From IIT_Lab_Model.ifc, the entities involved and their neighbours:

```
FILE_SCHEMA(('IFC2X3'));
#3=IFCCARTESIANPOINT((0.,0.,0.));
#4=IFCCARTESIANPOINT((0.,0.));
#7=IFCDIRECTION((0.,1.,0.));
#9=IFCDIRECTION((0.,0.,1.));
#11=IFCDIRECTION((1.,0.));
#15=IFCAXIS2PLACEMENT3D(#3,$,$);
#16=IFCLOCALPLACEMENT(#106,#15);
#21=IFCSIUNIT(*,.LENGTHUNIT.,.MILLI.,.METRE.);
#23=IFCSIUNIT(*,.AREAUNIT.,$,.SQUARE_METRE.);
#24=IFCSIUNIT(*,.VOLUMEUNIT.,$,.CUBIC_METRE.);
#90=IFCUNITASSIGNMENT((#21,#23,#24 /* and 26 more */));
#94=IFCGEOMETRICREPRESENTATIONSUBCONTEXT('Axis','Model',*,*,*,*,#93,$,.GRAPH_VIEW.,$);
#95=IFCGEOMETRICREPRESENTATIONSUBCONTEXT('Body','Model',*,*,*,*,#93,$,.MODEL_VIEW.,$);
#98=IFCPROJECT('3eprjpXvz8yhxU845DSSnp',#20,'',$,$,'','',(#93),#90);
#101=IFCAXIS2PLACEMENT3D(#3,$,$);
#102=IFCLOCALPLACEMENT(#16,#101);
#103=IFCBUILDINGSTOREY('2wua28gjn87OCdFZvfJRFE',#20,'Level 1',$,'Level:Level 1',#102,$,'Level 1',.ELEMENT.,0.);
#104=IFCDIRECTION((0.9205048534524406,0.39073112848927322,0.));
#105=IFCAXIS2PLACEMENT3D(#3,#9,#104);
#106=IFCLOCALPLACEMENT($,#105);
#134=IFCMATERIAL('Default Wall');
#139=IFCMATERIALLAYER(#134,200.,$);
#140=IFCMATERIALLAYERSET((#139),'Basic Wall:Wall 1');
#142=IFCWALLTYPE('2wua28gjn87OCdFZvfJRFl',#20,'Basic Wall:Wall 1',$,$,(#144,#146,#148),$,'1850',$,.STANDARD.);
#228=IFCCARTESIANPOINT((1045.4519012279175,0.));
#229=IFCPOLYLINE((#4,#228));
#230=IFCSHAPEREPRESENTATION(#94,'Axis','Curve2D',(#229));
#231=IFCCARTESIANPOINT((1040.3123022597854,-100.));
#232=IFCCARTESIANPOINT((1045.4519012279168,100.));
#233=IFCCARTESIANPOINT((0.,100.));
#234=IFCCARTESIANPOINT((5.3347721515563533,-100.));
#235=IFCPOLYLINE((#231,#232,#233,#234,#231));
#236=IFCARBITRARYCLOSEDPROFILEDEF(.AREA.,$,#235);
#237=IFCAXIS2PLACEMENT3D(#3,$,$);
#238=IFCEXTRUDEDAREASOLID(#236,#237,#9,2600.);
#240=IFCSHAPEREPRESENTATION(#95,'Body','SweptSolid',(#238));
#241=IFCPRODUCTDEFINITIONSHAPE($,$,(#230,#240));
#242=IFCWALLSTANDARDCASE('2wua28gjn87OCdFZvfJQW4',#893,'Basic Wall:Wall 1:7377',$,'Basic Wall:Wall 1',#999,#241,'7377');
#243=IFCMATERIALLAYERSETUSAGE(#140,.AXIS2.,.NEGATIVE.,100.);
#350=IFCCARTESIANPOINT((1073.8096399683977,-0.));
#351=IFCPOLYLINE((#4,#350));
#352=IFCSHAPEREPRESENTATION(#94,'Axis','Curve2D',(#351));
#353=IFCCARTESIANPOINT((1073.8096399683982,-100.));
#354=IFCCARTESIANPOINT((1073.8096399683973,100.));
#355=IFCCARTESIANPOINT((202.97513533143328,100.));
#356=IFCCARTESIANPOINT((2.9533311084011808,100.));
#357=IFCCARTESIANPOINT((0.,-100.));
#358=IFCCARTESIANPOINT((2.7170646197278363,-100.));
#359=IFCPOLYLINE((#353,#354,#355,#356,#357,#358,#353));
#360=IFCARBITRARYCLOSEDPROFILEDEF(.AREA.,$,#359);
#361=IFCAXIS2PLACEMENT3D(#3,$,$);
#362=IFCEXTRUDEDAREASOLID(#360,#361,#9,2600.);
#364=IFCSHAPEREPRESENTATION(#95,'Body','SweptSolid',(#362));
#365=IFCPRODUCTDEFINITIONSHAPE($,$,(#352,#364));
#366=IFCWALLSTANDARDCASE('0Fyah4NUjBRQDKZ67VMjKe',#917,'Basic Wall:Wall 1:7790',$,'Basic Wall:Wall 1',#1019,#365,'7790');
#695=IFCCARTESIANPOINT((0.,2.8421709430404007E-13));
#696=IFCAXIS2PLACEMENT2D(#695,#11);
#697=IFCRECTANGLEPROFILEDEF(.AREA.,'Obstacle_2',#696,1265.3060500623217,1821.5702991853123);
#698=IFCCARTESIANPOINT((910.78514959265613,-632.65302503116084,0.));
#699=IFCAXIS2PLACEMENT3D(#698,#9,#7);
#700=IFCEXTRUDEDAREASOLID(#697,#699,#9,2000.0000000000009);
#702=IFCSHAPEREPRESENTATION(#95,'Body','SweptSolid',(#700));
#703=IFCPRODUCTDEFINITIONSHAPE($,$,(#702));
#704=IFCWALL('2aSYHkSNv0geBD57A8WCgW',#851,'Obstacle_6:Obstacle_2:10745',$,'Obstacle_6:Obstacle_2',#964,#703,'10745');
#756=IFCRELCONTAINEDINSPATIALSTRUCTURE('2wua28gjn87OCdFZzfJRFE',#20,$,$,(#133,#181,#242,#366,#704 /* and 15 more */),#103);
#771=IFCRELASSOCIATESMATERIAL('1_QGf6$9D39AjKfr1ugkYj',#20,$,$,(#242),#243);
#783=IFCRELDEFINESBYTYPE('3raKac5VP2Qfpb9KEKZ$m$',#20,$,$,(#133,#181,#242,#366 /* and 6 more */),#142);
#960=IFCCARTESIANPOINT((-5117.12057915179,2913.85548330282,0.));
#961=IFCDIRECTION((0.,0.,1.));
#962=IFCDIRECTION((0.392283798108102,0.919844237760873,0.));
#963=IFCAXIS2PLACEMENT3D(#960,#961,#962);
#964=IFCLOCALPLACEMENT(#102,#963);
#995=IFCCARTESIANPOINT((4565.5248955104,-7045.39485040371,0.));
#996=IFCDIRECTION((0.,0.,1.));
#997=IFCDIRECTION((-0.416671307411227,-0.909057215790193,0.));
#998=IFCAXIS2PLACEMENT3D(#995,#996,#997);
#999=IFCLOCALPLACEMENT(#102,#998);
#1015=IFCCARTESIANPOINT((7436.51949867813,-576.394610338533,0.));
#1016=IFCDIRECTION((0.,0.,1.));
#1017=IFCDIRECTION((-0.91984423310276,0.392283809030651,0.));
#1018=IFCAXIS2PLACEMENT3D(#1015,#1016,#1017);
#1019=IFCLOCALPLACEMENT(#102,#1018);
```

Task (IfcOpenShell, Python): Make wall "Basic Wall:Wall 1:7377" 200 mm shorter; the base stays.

```python
import ifcopenshell
import ifcopenshell.geom
import ifcopenshell.util.representation
import ifcopenshell.util.shape
import ifcopenshell.util.unit

model = ifcopenshell.open("IIT_Lab_Model.ifc")
unit_scale = ifcopenshell.util.unit.calculate_unit_scale(model)
settings = ifcopenshell.geom.settings()


def volume(element):
    """Net volume in cubic metres, openings subtracted."""
    shape = ifcopenshell.geom.create_shape(settings, element)
    return ifcopenshell.util.shape.get_volume(shape.geometry)


wall = model.by_guid("2wua28gjn87OCdFZvfJQW4")
before = volume(wall)

body = ifcopenshell.util.representation.get_representation(wall, "Model", "Body")
solid = body.Items[0]
old_height = solid.Depth
solid.Depth -= 0.2 / unit_scale
after = volume(wall)

print(f"height {old_height:g} -> {solid.Depth:g}, volume {before:.3f} -> {after:.3f} m3")

model.write("IIT_Lab_Model_rev.ifc")
```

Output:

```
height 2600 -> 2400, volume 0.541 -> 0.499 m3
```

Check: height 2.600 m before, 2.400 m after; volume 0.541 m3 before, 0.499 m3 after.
